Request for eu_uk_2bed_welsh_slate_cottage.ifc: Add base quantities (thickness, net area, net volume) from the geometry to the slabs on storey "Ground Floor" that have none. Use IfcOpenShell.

First a look at what the model holds.

```python
import ifcopenshell
import ifcopenshell.util.element
import ifcopenshell.util.unit

model = ifcopenshell.open("eu_uk_2bed_welsh_slate_cottage.ifc")
print(model.schema)
for unit_type in ("LENGTHUNIT", "AREAUNIT", "VOLUMEUNIT"):
    print(unit_type, ifcopenshell.util.unit.calculate_unit_scale(model, unit_type))
storey = next(s for s in model.by_type("IfcBuildingStorey") if s.Name == "Ground Floor")
slabs = [e for e in ifcopenshell.util.element.get_decomposition(storey) if e.is_a("IfcSlab")]
for e in sorted(slabs, key=lambda e: e.id()):
    print(e.id(), e.is_a(), e.Name, list(ifcopenshell.util.element.get_psets(e, qtos_only=True)), sep=" | ")
```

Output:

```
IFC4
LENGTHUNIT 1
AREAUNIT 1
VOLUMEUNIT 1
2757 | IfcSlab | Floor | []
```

```python
import ifcopenshell
import ifcopenshell.api.pset
import ifcopenshell.geom
import ifcopenshell.util.element
import ifcopenshell.util.shape
import ifcopenshell.util.unit

model = ifcopenshell.open("eu_uk_2bed_welsh_slate_cottage.ifc")
unit_scale = ifcopenshell.util.unit.calculate_unit_scale(model)
area_scale = ifcopenshell.util.unit.calculate_unit_scale(model, "AREAUNIT")
volume_scale = ifcopenshell.util.unit.calculate_unit_scale(model, "VOLUMEUNIT")
settings = ifcopenshell.geom.settings()

storey = next(s for s in model.by_type("IfcBuildingStorey") if s.Name == "Ground Floor")
slabs = [e for e in ifcopenshell.util.element.get_decomposition(storey) if e.is_a("IfcSlab")]

for e in sorted(slabs, key=lambda e: e.id()):
    if ifcopenshell.util.element.get_psets(e, qtos_only=True, should_inherit=False):
        continue
    # Geometry comes back in metres, in the element's own axes.
    shape = ifcopenshell.geom.create_shape(settings, e)
    values = {
        "Width": ifcopenshell.util.shape.get_z(shape.geometry) / unit_scale,
        "NetArea": ifcopenshell.util.shape.get_footprint_area(shape.geometry) / area_scale,
        "NetVolume": ifcopenshell.util.shape.get_volume(shape.geometry) / volume_scale,
    }
    qto = ifcopenshell.api.pset.add_qto(model, product=e, name="Qto_SlabBaseQuantities")
    ifcopenshell.api.pset.edit_qto(model, qto=qto, properties=values)
    print(e.id(), {k: round(v, 3) for k, v in values.items()})

model.write("eu_uk_2bed_welsh_slate_cottage_updated.ifc")
```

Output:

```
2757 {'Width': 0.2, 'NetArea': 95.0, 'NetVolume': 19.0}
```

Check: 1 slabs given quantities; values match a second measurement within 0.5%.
